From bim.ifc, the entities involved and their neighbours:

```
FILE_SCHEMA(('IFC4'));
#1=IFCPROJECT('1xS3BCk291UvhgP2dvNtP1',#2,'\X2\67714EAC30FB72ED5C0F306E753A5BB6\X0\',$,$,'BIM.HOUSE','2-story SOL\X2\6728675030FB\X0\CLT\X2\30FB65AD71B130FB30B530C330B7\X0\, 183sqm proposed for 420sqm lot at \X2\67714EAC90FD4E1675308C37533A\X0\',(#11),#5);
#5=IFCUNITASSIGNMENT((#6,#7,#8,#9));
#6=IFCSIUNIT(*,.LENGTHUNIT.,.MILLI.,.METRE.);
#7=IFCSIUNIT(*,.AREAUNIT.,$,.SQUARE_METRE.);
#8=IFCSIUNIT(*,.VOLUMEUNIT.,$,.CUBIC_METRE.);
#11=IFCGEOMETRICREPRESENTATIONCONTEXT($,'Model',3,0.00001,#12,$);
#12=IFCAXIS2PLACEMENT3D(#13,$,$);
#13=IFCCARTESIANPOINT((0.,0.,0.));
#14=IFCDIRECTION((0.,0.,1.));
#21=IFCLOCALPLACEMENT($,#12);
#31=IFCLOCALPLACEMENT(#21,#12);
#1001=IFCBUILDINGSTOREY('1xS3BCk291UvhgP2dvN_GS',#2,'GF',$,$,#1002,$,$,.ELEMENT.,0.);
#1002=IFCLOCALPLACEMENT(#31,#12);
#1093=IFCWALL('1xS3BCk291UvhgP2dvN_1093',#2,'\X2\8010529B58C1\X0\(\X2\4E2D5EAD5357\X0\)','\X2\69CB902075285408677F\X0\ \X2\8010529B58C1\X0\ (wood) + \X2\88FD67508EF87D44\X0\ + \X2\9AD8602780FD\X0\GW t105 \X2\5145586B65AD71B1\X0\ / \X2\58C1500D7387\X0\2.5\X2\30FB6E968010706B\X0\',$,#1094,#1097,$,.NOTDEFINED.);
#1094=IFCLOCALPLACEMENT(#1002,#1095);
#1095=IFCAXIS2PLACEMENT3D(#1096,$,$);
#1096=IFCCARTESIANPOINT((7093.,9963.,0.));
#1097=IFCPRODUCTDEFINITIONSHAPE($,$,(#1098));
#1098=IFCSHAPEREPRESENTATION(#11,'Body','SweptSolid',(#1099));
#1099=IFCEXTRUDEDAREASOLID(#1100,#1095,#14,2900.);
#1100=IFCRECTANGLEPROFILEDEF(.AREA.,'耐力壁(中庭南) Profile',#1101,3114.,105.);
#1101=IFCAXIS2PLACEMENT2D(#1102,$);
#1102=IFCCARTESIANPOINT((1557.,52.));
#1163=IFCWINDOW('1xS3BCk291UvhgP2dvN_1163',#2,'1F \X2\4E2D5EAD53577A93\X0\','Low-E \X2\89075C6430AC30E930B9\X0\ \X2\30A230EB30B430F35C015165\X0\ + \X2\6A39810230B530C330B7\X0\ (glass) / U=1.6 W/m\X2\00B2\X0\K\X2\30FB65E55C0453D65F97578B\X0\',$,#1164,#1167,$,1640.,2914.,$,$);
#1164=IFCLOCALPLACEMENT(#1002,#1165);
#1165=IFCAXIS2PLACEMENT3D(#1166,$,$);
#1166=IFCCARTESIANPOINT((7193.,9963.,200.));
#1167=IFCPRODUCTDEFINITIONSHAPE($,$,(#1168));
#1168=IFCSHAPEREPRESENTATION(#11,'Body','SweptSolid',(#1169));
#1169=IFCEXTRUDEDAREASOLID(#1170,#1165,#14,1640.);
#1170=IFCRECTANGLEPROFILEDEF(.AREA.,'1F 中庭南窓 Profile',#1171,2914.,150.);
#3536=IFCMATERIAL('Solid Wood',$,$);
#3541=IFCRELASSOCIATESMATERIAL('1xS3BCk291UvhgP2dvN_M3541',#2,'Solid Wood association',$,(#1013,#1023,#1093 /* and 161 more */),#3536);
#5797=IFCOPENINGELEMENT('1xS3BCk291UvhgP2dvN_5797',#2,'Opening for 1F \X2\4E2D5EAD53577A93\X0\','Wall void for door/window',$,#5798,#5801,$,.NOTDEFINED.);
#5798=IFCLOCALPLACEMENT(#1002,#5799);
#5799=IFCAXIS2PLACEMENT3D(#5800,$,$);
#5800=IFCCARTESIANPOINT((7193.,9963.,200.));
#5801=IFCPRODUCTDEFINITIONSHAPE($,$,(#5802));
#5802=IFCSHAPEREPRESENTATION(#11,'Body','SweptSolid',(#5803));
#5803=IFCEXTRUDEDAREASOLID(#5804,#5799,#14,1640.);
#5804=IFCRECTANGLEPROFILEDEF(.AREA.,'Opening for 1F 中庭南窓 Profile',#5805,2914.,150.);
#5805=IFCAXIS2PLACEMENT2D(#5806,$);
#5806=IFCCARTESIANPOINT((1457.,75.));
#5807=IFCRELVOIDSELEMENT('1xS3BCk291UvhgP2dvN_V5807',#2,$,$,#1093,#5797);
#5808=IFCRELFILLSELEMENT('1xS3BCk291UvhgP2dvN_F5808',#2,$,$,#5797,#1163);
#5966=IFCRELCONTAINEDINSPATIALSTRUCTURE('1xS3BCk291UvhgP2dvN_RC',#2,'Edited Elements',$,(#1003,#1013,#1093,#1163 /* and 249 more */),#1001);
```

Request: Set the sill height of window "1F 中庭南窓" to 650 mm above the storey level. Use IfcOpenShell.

```python
import numpy as np
import ifcopenshell
import ifcopenshell.api.geometry
import ifcopenshell.geom
import ifcopenshell.util.element
import ifcopenshell.util.placement
import ifcopenshell.util.shape
import ifcopenshell.util.unit

model = ifcopenshell.open("bim.ifc")
unit_scale = ifcopenshell.util.unit.calculate_unit_scale(model)

window = model.by_guid("1xS3BCk291UvhgP2dvN_1163")
opening = window.FillsVoids[0].RelatingOpeningElement
storey = ifcopenshell.util.element.get_container(window, ifc_class="IfcBuildingStorey")
level = ifcopenshell.util.placement.get_local_placement(storey.ObjectPlacement)[2, 3]

# The opening's origin need not be at the sill, so measure its lowest point.
shape = ifcopenshell.geom.create_shape(ifcopenshell.geom.settings(), opening)
bottom = ifcopenshell.util.shape.get_shape_bottom_elevation(shape, shape.geometry) / unit_scale
dz = level + 650.0 - bottom

shift = np.array([0.0, 0.0, dz])
# The window is not placed relative to its opening, so move both.
for product in (opening, window):
    matrix = ifcopenshell.util.placement.get_local_placement(product.ObjectPlacement)
    matrix[:3, 3] += shift
    ifcopenshell.api.geometry.edit_object_placement(model, product=product, matrix=matrix, is_si=False)

print(f"moved by {dz * unit_scale:+.3f} m")

model.write("bim_updated.ifc")
```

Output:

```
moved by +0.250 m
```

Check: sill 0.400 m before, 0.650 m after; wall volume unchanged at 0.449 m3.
